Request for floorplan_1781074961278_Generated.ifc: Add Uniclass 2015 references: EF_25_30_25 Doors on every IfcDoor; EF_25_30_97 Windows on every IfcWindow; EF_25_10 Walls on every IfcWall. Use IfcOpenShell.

First a look at what the model holds.

```python
import ifcopenshell

model = ifcopenshell.open("floorplan_1781074961278_Generated.ifc")
print(model.schema)
print("classifications:", [c.Name for c in model.by_type("IfcClassification")])
for ifc_class in ("IfcDoor", "IfcRoof", "IfcStair", "IfcWall", "IfcWindow"):
    print(ifc_class, len(model.by_type(ifc_class)))
```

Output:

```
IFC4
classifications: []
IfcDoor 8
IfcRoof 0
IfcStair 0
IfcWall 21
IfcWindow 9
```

```python
import ifcopenshell
import ifcopenshell.api.classification

model = ifcopenshell.open("floorplan_1781074961278_Generated.ifc")

system = ifcopenshell.api.classification.add_classification(model, classification="Uniclass 2015")

codes = {
    "IfcDoor": ("EF_25_30_25", "Doors"),
    "IfcWindow": ("EF_25_30_97", "Windows"),
    "IfcWall": ("EF_25_10", "Walls"),
}
for ifc_class, (code, name) in codes.items():
    products = model.by_type(ifc_class)
    ifcopenshell.api.classification.add_reference(
        model, products=products, classification=system, identification=code, name=name
    )
    print(code, len(products))

model.write("floorplan_1781074961278_Generated_updated.ifc")
```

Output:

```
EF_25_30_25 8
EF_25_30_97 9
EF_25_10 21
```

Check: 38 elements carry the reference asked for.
